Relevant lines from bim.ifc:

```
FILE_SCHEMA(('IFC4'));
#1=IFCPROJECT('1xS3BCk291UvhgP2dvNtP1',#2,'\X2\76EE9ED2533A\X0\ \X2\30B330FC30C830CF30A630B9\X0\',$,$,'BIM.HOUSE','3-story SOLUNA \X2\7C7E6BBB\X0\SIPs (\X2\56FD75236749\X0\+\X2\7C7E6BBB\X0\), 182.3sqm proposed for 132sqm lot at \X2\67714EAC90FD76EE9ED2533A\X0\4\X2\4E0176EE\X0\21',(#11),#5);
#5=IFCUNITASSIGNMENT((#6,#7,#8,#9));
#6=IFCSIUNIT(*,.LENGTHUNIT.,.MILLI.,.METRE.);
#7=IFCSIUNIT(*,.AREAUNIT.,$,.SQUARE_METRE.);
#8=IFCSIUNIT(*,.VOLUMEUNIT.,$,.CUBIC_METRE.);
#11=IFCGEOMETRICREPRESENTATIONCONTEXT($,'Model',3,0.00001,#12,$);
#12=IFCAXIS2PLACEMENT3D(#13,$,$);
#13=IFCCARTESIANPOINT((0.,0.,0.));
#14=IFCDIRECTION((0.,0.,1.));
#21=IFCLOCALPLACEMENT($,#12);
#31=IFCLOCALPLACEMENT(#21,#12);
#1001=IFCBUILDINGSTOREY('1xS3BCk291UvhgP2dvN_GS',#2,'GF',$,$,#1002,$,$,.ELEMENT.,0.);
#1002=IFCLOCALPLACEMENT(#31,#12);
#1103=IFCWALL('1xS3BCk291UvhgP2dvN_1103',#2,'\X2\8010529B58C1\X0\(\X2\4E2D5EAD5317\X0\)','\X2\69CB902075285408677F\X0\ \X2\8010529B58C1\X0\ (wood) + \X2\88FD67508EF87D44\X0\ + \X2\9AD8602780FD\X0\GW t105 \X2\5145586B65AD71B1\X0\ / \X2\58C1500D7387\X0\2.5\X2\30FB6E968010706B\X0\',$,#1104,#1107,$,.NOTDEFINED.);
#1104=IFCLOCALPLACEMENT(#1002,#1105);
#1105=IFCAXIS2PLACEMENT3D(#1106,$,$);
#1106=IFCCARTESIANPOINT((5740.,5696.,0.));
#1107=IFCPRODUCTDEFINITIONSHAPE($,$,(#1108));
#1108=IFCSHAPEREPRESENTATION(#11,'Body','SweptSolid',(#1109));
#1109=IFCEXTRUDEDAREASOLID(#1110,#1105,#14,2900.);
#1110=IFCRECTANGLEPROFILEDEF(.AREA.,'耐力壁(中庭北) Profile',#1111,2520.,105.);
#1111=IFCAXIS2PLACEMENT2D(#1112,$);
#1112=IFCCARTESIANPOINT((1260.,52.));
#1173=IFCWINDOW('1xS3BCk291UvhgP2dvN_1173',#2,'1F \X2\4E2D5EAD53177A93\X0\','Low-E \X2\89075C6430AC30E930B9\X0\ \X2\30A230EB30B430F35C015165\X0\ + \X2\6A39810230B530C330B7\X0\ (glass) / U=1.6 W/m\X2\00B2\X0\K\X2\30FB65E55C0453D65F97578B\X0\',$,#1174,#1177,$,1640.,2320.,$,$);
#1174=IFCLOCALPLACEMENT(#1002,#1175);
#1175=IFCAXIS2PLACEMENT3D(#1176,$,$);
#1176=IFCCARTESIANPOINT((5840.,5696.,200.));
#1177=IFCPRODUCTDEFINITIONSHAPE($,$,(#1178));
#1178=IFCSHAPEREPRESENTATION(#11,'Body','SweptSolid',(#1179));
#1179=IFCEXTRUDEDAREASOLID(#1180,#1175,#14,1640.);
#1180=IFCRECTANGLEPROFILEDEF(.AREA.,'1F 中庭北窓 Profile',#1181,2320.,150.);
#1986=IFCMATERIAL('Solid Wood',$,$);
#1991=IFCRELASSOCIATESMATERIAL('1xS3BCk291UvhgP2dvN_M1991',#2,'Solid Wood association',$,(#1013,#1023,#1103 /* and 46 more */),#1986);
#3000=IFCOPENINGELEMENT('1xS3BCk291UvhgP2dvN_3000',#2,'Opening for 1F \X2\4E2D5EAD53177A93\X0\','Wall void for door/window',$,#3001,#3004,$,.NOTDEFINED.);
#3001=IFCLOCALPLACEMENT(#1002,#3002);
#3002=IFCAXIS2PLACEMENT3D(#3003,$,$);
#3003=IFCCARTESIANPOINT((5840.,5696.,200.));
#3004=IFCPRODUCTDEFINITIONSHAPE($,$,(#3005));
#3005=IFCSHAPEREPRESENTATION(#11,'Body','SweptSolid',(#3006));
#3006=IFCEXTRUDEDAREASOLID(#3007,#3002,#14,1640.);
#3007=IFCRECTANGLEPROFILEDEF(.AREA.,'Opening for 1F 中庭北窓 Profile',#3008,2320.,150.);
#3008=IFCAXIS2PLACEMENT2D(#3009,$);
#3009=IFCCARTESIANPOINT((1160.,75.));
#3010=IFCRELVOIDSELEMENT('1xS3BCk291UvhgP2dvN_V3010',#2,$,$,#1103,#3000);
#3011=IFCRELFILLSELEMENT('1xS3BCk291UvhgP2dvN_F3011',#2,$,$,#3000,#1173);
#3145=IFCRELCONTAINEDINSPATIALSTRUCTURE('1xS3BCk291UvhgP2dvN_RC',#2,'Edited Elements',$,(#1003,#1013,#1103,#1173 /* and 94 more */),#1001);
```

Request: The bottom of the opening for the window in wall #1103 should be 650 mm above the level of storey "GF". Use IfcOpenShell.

```python
import numpy as np
import ifcopenshell
import ifcopenshell.api.geometry
import ifcopenshell.geom
import ifcopenshell.util.element
import ifcopenshell.util.placement
import ifcopenshell.util.shape
import ifcopenshell.util.unit

model = ifcopenshell.open("bim.ifc")
unit_scale = ifcopenshell.util.unit.calculate_unit_scale(model)

window = model.by_id(1173)
opening = window.FillsVoids[0].RelatingOpeningElement
storey = ifcopenshell.util.element.get_container(window, ifc_class="IfcBuildingStorey")
level = ifcopenshell.util.placement.get_local_placement(storey.ObjectPlacement)[2, 3]

# The opening's origin need not be at the sill, so measure its lowest point.
shape = ifcopenshell.geom.create_shape(ifcopenshell.geom.settings(), opening)
bottom = ifcopenshell.util.shape.get_shape_bottom_elevation(shape, shape.geometry) / unit_scale
dz = level + 0.65 / unit_scale - bottom

shift = np.array([0.0, 0.0, dz])
# The window is not placed relative to its opening, so move both.
for product in (opening, window):
    matrix = ifcopenshell.util.placement.get_local_placement(product.ObjectPlacement)
    matrix[:3, 3] += shift
    ifcopenshell.api.geometry.edit_object_placement(model, product=product, matrix=matrix, is_si=False)

print(f"moved by {dz * unit_scale:+.3f} m")

model.write("bim_updated.ifc")
```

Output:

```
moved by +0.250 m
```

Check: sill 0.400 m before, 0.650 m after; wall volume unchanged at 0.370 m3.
